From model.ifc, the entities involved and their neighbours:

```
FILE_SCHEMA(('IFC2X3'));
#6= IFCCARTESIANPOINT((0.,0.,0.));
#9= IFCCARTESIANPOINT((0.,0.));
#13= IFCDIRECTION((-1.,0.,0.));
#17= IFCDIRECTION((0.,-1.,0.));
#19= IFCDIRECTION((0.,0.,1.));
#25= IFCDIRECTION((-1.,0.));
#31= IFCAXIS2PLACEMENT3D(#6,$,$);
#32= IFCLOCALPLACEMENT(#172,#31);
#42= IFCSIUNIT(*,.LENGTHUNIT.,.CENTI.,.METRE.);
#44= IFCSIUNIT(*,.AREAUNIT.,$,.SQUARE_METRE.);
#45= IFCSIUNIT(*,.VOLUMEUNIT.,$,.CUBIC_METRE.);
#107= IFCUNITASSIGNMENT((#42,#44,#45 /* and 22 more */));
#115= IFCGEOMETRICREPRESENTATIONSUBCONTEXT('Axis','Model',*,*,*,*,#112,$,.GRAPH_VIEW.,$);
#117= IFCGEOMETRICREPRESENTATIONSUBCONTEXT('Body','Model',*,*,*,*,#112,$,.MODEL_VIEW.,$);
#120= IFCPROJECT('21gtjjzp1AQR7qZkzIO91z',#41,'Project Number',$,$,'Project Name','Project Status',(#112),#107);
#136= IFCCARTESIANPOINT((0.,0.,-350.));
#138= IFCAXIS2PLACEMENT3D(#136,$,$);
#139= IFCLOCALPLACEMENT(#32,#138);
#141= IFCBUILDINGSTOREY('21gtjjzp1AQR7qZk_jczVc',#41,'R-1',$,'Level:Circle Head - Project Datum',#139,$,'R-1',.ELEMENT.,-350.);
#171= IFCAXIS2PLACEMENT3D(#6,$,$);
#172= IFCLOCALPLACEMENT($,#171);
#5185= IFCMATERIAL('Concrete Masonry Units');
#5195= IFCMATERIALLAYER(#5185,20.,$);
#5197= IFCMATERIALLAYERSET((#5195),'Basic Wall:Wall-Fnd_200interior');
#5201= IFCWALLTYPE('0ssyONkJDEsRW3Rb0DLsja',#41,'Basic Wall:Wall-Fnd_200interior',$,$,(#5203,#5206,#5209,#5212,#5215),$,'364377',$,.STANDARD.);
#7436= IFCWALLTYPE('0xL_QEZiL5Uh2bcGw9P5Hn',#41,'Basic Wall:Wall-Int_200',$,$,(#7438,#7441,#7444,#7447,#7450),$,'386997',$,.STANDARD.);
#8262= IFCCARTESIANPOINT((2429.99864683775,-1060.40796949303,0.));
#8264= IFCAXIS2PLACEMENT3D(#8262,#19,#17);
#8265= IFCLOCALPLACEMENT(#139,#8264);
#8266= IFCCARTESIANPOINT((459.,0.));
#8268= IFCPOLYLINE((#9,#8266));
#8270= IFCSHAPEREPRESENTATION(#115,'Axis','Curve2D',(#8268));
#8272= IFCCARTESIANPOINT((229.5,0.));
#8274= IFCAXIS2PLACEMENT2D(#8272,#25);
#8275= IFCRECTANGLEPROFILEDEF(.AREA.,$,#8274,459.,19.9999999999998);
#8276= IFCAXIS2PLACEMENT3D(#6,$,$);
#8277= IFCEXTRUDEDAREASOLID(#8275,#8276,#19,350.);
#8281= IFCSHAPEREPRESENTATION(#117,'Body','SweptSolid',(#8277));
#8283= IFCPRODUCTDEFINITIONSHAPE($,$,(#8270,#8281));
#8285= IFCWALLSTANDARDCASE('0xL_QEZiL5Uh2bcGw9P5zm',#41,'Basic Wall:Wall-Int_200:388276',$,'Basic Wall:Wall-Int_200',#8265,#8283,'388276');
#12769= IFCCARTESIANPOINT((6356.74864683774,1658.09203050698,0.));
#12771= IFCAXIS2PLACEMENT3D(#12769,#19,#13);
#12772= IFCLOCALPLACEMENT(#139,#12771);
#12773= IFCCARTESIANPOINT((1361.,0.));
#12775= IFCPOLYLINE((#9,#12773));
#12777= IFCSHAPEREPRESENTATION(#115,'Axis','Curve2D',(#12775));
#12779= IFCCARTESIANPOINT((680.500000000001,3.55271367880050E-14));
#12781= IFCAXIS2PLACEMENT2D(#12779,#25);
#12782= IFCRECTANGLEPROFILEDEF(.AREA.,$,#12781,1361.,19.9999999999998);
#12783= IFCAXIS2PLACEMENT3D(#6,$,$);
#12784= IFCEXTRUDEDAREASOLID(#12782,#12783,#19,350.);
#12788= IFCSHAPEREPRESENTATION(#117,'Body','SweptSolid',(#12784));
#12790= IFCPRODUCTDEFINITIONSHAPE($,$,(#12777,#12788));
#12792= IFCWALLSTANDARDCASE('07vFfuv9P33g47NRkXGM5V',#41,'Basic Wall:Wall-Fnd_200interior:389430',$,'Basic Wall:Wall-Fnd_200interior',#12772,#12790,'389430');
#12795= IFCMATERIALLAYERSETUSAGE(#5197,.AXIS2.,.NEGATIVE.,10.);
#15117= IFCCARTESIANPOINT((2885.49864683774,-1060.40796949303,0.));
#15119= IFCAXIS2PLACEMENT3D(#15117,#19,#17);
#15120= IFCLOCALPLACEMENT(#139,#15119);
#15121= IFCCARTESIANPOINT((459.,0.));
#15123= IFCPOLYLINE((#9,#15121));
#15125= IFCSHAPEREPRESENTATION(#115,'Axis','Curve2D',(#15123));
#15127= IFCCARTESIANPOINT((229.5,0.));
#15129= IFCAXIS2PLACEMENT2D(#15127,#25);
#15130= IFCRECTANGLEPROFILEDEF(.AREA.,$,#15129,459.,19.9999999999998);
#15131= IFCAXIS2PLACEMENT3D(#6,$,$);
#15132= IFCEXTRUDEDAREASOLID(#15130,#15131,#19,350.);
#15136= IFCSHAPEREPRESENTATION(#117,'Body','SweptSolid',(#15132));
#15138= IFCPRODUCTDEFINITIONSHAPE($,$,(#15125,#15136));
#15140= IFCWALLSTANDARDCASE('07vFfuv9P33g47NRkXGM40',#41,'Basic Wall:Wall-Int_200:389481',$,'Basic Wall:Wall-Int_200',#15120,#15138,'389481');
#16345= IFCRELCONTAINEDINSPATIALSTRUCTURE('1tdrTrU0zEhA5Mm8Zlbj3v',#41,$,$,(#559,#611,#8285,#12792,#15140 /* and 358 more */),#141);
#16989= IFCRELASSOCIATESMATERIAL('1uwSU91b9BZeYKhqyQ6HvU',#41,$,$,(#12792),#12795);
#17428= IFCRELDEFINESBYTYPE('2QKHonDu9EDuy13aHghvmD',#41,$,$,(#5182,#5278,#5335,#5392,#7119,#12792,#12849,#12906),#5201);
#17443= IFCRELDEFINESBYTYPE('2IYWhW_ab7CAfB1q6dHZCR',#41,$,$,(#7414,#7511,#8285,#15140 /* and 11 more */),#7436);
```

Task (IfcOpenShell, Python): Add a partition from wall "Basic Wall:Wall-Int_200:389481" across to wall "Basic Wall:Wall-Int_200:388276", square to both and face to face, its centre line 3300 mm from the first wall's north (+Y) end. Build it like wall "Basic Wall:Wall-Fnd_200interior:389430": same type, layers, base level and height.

```python
import numpy as np
import ifcopenshell
import ifcopenshell.api.geometry
import ifcopenshell.api.material
import ifcopenshell.api.pset
import ifcopenshell.api.root
import ifcopenshell.api.spatial
import ifcopenshell.api.type
import ifcopenshell.geom
import ifcopenshell.util.element
import ifcopenshell.util.placement
import ifcopenshell.util.representation
import ifcopenshell.util.shape
import ifcopenshell.util.unit

model = ifcopenshell.open("model.ifc")
unit_scale = ifcopenshell.util.unit.calculate_unit_scale(model)
settings = ifcopenshell.geom.settings()
settings.set("use-world-coords", True)

start_wall = model.by_guid("07vFfuv9P33g47NRkXGM40")
end_wall = model.by_guid("0xL_QEZiL5Uh2bcGw9P5zm")
like = model.by_guid("07vFfuv9P33g47NRkXGM5V")
matrix = ifcopenshell.util.placement.get_local_placement(start_wall.ObjectPlacement)
matrix[:3, 3] *= unit_scale


def extent(element):
    """Bounding box in the first wall's axes, in metres."""
    shape = ifcopenshell.geom.create_shape(settings, element)
    points = (ifcopenshell.util.shape.get_vertices(shape.geometry) - matrix[:3, 3]) @ matrix[:3, :3]
    return points.min(axis=0), points.max(axis=0)


y_start = extent(start_wall)[0][1]
y_end = extent(end_wall)[1][1]
like_min, like_max = extent(like)
length, height = float(abs(y_end - y_start)), float(like_max[2] - like_min[2])
layer_set = ifcopenshell.util.element.get_material(like, should_skip_usage=True)
thickness = sum(layer.LayerThickness for layer in layer_set.MaterialLayers) * unit_scale

wall = ifcopenshell.api.root.create_entity(model, ifc_class="IfcWallStandardCase", name="New partition")
storey = ifcopenshell.util.element.get_container(like)
ifcopenshell.api.spatial.assign_container(model, products=[wall], relating_structure=storey)
ifcopenshell.api.type.assign_type(
    model, related_objects=[wall], relating_type=ifcopenshell.util.element.get_type(like), should_map_representations=False
)
rel = ifcopenshell.api.material.assign_material(
    model, products=[wall], type="IfcMaterialLayerSetUsage", material=layer_set
)
rel.RelatingMaterial.OffsetFromReferenceLine = -thickness / 2 / unit_scale
pset = ifcopenshell.api.pset.add_pset(model, product=wall, name="Pset_WallCommon")
ifcopenshell.api.pset.edit_pset(model, pset=pset, properties={"IsExternal": False, "LoadBearing": False})

# The axis runs down the middle of the wall.
axis = ifcopenshell.api.geometry.add_axis_representation(
    model, context=ifcopenshell.util.representation.get_context(model, "Model", "Axis"), axis=[(0.0, 0.0), (length, 0.0)]
)
body = ifcopenshell.api.geometry.add_wall_representation(
    model,
    context=ifcopenshell.util.representation.get_context(model, "Model", "Body", "MODEL_VIEW"),
    length=length,
    height=height,
    thickness=thickness,
    offset=-thickness / 2,
)
for representation in (axis, body):
    ifcopenshell.api.geometry.assign_representation(model, product=wall, representation=representation)

placement = matrix @ ifcopenshell.util.placement.rotation(-90, "Z")
placement[:, 3] = matrix @ np.array([extent(start_wall)[0][0] + 3.3, y_start, like_min[2], 1.0])
ifcopenshell.api.geometry.edit_object_placement(model, product=wall, matrix=placement)

print(f"partition {length:.3f} m long, {height:.3f} m high, {thickness:.3f} m thick")

model.write("model_rev.ifc")
```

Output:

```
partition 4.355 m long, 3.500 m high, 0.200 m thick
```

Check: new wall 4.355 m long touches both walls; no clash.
